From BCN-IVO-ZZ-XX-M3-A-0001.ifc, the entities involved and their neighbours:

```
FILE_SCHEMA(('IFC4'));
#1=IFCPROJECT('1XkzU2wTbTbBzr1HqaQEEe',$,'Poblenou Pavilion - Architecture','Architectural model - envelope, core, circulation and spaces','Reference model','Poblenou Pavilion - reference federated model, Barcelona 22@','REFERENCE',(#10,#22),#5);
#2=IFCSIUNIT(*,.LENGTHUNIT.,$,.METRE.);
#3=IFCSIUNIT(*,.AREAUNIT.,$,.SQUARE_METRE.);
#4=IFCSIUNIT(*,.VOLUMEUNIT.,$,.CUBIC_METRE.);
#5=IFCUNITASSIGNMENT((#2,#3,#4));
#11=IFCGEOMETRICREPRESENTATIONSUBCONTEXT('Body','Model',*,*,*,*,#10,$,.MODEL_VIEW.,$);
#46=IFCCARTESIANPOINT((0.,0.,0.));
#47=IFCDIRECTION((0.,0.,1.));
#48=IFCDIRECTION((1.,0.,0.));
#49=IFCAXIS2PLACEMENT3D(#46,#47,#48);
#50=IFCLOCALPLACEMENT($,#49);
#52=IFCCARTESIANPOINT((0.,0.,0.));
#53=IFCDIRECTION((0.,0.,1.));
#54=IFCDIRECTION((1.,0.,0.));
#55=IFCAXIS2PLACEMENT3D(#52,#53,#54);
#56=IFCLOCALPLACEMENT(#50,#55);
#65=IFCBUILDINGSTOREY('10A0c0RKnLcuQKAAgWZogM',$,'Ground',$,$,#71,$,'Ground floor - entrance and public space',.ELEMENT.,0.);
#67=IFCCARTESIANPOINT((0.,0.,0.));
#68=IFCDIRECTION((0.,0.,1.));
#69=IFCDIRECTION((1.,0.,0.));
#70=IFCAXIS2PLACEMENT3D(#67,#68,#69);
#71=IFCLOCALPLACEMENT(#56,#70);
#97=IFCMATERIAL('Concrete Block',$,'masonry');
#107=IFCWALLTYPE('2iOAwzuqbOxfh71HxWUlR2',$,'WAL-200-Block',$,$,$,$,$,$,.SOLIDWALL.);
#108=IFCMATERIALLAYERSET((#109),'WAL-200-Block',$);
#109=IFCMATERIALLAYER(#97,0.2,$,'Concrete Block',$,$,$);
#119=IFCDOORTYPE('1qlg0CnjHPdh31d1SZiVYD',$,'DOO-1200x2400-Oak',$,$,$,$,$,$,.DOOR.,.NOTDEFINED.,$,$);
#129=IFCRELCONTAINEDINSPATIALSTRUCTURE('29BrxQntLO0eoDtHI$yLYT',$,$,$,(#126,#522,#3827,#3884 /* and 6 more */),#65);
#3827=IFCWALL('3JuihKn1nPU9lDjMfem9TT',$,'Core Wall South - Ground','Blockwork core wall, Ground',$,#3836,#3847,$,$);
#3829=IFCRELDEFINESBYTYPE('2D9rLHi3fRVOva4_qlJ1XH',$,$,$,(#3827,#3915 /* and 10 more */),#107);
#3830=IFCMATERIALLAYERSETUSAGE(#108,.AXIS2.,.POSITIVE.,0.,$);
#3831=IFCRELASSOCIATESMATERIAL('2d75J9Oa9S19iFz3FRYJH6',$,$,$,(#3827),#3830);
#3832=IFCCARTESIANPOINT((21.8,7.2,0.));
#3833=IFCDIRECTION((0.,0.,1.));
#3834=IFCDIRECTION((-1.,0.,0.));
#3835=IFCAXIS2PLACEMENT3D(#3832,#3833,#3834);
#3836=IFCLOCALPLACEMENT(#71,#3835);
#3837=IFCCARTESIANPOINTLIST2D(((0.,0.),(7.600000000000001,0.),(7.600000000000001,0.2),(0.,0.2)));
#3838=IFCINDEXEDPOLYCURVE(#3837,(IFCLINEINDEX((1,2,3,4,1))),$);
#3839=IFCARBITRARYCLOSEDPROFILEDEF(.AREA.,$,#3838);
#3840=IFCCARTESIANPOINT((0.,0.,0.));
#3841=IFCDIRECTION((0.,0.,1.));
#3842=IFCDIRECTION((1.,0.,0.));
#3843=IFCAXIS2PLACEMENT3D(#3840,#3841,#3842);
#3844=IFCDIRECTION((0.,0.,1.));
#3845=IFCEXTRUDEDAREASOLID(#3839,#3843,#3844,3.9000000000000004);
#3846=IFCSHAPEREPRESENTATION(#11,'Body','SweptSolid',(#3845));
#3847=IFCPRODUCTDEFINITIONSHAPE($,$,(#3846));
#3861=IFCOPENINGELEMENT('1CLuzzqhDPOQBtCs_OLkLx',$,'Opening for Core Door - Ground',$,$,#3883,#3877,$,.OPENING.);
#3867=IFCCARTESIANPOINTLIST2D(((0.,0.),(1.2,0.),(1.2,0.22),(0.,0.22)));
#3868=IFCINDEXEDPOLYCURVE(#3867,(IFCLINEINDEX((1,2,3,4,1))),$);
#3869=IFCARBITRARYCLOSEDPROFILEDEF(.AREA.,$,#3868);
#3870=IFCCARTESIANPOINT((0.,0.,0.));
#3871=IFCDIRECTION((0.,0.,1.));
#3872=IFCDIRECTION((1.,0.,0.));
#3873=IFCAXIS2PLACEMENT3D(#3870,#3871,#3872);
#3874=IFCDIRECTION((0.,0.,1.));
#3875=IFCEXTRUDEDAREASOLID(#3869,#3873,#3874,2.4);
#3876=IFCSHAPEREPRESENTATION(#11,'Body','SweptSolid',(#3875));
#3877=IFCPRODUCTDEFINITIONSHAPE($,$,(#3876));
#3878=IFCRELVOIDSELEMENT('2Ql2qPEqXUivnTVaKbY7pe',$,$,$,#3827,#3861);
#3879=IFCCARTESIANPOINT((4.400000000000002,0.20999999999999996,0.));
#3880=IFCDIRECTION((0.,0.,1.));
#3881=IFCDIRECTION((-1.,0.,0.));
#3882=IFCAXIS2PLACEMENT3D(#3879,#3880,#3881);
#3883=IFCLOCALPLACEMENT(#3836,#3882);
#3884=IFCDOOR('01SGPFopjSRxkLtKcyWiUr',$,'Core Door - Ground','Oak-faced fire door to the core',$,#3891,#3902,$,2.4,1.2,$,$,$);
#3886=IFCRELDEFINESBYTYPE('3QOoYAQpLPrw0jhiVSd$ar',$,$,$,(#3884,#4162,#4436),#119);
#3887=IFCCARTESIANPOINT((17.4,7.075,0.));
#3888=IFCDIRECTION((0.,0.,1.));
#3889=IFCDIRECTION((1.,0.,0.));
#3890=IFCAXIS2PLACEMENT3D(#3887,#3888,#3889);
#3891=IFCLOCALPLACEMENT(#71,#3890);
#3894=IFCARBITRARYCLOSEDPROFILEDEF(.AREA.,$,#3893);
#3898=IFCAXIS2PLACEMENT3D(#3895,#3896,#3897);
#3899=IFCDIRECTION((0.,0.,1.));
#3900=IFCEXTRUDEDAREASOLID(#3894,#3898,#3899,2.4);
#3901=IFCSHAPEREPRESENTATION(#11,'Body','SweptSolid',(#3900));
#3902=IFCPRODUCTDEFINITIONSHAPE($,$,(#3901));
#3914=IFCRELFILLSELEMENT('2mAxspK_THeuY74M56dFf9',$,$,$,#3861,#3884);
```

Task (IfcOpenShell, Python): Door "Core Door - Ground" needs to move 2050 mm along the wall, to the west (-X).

```python
import ifcopenshell
import ifcopenshell.api.geometry
import ifcopenshell.util.placement
import ifcopenshell.util.unit

model = ifcopenshell.open("BCN-IVO-ZZ-XX-M3-A-0001.ifc")
unit_scale = ifcopenshell.util.unit.calculate_unit_scale(model)

door = model.by_guid("01SGPFopjSRxkLtKcyWiUr")
opening = door.FillsVoids[0].RelatingOpeningElement
wall = opening.VoidsElements[0].RelatingBuildingElement

wall_matrix = ifcopenshell.util.placement.get_local_placement(wall.ObjectPlacement)
shift = wall_matrix[:3, 0] * 2.05 / unit_scale
before = ifcopenshell.util.placement.get_local_placement(door.ObjectPlacement)[:3, 3].copy()

# The door is not placed relative to its opening, so move both.
for product in (opening, door):
    matrix = ifcopenshell.util.placement.get_local_placement(product.ObjectPlacement)
    matrix[:3, 3] += shift
    ifcopenshell.api.geometry.edit_object_placement(model, product=product, matrix=matrix, is_si=False)

after = ifcopenshell.util.placement.get_local_placement(door.ObjectPlacement)[:3, 3]
print("door moved by", (after - before).round(3) + 0.0)

model.write("BCN-IVO-ZZ-XX-M3-A-0001_rev.ifc")
```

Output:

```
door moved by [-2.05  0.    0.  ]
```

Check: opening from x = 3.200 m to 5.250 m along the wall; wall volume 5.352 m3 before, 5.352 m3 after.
